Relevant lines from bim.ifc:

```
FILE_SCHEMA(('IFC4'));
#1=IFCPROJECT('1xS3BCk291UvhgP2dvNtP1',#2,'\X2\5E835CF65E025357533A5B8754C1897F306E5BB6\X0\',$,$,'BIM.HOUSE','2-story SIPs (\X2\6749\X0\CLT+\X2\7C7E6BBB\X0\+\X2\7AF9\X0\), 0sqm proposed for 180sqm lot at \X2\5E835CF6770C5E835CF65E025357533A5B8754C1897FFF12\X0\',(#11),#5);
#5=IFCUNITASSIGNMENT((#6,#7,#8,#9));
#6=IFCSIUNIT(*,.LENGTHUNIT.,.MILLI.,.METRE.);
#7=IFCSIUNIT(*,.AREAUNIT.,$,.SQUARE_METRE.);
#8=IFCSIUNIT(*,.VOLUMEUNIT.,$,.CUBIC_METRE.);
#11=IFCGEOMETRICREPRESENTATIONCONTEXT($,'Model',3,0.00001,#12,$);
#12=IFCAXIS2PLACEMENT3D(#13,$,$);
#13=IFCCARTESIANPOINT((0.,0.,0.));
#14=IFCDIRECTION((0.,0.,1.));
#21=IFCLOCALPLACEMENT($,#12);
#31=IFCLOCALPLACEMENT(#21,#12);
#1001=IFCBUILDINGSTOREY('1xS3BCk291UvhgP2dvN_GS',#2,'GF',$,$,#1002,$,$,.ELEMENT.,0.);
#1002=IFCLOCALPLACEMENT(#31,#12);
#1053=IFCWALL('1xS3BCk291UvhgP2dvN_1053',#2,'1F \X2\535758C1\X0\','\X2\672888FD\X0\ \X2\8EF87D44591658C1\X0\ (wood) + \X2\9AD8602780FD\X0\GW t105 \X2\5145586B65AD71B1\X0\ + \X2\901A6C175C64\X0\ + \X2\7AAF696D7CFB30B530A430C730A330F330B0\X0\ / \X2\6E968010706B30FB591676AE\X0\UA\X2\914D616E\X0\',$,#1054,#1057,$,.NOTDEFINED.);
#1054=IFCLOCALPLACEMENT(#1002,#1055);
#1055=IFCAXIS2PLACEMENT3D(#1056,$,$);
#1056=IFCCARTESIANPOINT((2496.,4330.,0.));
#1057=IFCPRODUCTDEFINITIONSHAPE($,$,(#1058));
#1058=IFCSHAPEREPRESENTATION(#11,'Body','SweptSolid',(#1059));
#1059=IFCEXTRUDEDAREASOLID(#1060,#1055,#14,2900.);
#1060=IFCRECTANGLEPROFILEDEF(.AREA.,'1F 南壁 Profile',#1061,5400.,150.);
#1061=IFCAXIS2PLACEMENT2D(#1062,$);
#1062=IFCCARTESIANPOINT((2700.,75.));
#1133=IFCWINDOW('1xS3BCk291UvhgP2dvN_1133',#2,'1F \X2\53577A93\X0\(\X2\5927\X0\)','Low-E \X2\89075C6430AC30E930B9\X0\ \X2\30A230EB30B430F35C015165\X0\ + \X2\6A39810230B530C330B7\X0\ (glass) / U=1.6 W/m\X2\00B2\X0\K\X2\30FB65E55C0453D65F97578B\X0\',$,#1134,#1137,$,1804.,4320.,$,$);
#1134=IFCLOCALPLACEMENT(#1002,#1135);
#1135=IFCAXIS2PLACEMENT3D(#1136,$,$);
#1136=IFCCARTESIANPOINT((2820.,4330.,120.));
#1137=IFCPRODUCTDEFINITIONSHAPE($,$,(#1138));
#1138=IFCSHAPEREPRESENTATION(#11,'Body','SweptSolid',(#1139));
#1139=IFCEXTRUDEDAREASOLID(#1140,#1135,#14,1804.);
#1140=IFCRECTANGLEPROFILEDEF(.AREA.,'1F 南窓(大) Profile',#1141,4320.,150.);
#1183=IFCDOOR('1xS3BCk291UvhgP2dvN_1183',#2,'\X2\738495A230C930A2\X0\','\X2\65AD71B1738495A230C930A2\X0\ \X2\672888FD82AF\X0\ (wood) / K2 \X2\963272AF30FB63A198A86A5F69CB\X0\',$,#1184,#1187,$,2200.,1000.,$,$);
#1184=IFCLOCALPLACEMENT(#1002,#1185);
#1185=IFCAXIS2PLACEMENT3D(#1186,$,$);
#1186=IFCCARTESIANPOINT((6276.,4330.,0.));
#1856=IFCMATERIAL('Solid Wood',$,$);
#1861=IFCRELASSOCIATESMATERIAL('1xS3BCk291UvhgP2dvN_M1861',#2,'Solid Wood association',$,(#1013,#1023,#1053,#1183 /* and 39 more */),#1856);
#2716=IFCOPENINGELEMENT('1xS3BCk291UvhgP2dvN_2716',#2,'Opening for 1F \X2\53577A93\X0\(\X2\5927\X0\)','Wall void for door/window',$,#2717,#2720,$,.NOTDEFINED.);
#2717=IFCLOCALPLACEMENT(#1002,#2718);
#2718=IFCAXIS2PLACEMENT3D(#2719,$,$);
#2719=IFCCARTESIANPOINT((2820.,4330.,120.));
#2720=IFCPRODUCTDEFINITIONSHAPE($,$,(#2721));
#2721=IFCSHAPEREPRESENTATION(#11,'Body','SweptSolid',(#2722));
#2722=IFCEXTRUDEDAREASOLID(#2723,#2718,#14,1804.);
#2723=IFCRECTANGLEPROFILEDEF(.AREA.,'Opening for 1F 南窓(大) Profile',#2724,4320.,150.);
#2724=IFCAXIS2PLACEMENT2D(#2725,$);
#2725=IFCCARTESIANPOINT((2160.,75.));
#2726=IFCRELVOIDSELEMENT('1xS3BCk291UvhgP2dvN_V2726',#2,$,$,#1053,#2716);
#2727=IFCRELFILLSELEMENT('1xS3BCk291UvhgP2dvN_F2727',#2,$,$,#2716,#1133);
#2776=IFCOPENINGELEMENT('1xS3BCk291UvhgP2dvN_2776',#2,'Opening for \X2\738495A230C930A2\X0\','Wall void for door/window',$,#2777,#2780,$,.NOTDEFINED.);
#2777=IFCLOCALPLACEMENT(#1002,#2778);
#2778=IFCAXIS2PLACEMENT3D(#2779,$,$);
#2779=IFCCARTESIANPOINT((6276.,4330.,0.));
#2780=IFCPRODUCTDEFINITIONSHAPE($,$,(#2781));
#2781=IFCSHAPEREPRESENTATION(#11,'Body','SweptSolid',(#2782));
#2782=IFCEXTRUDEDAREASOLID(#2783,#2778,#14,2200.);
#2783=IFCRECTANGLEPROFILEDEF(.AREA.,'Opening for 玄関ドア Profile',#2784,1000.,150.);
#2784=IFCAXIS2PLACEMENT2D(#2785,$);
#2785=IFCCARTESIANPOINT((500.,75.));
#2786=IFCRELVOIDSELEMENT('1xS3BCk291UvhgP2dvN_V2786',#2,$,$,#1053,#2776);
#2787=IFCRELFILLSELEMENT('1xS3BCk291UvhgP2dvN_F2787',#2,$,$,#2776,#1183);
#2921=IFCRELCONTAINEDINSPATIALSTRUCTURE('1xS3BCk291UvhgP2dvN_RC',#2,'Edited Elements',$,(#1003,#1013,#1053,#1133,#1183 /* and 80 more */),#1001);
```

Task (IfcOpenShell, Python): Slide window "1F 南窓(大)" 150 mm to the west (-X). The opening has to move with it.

```python
import ifcopenshell
import ifcopenshell.api.geometry
import ifcopenshell.util.placement

model = ifcopenshell.open("bim.ifc")

window = model.by_guid("1xS3BCk291UvhgP2dvN_1133")
opening = window.FillsVoids[0].RelatingOpeningElement
wall = opening.VoidsElements[0].RelatingBuildingElement

wall_matrix = ifcopenshell.util.placement.get_local_placement(wall.ObjectPlacement)
shift = wall_matrix[:3, 0] * -150.0
before = ifcopenshell.util.placement.get_local_placement(window.ObjectPlacement)[:3, 3].copy()

# The window is not placed relative to its opening, so move both.
for product in (opening, window):
    matrix = ifcopenshell.util.placement.get_local_placement(product.ObjectPlacement)
    matrix[:3, 3] += shift
    ifcopenshell.api.geometry.edit_object_placement(model, product=product, matrix=matrix, is_si=False)

after = ifcopenshell.util.placement.get_local_placement(window.ObjectPlacement)[:3, 3]
print("window moved by", (after - before).round(3) + 0.0)

model.write("bim_v2.ifc")
```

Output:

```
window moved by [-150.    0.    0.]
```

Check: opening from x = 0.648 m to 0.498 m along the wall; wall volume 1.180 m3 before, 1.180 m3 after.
